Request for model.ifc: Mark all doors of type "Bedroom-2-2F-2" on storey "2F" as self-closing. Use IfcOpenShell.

First a look at what the model holds.

```python
import ifcopenshell
import ifcopenshell.util.element

model = ifcopenshell.open("model.ifc")
print(model.schema)
storey = next(s for s in model.by_type("IfcBuildingStorey") if s.Name == "2F")
doors = [e for e in ifcopenshell.util.element.get_decomposition(storey) if e.is_a("IfcDoor")]
seen = {}
for e in doors:
    element_type = ifcopenshell.util.element.get_type(e)
    key = (element_type.Name if element_type != e and element_type else None, ifcopenshell.util.element.get_pset(e, "Pset_DoorCommon", "SelfClosing"))
    seen[key] = seen.get(key, 0) + 1
for (name, value), count in sorted(seen.items(), key=str):
    print(count, "x", name, "|", value)
```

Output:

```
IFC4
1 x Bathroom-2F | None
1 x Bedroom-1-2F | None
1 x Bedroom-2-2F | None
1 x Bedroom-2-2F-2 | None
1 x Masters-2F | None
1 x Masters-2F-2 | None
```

```python
import ifcopenshell
import ifcopenshell.api.pset
import ifcopenshell.util.element

model = ifcopenshell.open("model.ifc")

storey = next(s for s in model.by_type("IfcBuildingStorey") if s.Name == "2F")
doors = [e for e in ifcopenshell.util.element.get_decomposition(storey) if e.is_a("IfcDoor")]

count = 0
for e in doors:
    element_type = ifcopenshell.util.element.get_type(e)
    if element_type in (None, e) or element_type.Name != "Bedroom-2-2F-2":
        continue
    # add_pset returns the element's existing set when there is one.
    pset = ifcopenshell.api.pset.add_pset(model, product=e, name="Pset_DoorCommon")
    ifcopenshell.api.pset.edit_pset(model, pset=pset, properties={"SelfClosing": True})
    count += 1

print(count, "doors updated")

model.write("model_rev.ifc")
```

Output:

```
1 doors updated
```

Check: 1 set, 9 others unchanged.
